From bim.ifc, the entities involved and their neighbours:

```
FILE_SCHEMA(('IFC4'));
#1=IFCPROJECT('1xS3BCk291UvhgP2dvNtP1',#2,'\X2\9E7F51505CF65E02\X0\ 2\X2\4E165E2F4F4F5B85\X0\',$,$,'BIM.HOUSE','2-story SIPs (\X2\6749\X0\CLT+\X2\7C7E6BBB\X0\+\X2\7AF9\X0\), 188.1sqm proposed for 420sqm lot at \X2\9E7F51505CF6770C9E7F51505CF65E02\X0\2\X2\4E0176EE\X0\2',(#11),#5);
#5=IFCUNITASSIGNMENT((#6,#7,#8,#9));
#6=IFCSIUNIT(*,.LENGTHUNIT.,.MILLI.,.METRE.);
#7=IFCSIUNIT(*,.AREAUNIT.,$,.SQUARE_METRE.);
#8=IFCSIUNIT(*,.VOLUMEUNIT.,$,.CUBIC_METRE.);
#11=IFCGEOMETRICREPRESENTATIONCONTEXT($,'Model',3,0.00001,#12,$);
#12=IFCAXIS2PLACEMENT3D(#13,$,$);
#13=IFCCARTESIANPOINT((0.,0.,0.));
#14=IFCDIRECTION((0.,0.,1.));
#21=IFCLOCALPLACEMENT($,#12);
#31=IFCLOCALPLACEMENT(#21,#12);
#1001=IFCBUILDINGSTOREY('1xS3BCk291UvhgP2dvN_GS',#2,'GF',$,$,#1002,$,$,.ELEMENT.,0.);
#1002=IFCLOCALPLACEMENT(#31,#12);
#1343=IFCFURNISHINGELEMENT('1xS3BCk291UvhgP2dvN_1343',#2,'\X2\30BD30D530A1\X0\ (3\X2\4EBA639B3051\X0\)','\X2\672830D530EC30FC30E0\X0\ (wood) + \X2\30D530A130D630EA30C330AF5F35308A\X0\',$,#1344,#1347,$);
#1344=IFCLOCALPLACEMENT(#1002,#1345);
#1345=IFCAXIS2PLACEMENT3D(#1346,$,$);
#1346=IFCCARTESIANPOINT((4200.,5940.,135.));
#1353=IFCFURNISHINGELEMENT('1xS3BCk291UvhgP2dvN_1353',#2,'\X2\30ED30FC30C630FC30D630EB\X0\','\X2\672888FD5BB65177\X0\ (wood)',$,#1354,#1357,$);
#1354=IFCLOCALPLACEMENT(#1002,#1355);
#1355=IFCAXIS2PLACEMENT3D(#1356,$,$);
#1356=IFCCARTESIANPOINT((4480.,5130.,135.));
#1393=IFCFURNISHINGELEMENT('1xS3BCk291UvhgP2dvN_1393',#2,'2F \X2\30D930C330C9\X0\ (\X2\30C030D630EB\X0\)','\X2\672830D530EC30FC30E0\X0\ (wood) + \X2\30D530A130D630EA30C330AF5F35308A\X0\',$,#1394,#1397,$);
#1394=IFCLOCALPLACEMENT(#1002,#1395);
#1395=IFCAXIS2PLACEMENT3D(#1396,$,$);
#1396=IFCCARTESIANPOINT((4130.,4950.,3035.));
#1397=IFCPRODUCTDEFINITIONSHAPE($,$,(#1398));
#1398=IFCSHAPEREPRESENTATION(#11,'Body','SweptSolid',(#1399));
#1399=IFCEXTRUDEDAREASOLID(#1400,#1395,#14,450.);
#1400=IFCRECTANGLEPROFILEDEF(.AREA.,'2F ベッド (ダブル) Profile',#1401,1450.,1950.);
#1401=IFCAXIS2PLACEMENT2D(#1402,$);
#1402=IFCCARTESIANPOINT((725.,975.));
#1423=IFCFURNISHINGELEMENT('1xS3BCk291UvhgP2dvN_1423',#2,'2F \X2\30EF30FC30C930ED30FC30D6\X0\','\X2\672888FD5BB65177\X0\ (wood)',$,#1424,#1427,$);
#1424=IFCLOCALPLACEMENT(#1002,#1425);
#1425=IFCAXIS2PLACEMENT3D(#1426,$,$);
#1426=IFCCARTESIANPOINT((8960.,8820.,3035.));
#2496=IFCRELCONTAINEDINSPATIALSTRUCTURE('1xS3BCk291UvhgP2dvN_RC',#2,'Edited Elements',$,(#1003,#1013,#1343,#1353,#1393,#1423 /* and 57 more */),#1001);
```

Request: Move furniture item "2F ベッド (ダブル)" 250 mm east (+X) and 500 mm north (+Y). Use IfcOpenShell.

```python
import ifcopenshell
import ifcopenshell.api.geometry
import ifcopenshell.util.placement

model = ifcopenshell.open("bim.ifc")

item = model.by_id(1393)
matrix = ifcopenshell.util.placement.get_local_placement(item.ObjectPlacement)
matrix[0, 3] += 250.0
matrix[1, 3] += 500.0
ifcopenshell.api.geometry.edit_object_placement(model, product=item, matrix=matrix, is_si=False)

print(ifcopenshell.util.placement.get_local_placement(item.ObjectPlacement).round(3) + 0.0)

model.write("bim_rev.ifc")
```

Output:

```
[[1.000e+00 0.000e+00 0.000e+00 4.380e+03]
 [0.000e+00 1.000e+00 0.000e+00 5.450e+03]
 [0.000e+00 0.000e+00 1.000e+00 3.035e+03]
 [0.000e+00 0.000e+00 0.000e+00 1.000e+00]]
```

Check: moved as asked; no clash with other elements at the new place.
